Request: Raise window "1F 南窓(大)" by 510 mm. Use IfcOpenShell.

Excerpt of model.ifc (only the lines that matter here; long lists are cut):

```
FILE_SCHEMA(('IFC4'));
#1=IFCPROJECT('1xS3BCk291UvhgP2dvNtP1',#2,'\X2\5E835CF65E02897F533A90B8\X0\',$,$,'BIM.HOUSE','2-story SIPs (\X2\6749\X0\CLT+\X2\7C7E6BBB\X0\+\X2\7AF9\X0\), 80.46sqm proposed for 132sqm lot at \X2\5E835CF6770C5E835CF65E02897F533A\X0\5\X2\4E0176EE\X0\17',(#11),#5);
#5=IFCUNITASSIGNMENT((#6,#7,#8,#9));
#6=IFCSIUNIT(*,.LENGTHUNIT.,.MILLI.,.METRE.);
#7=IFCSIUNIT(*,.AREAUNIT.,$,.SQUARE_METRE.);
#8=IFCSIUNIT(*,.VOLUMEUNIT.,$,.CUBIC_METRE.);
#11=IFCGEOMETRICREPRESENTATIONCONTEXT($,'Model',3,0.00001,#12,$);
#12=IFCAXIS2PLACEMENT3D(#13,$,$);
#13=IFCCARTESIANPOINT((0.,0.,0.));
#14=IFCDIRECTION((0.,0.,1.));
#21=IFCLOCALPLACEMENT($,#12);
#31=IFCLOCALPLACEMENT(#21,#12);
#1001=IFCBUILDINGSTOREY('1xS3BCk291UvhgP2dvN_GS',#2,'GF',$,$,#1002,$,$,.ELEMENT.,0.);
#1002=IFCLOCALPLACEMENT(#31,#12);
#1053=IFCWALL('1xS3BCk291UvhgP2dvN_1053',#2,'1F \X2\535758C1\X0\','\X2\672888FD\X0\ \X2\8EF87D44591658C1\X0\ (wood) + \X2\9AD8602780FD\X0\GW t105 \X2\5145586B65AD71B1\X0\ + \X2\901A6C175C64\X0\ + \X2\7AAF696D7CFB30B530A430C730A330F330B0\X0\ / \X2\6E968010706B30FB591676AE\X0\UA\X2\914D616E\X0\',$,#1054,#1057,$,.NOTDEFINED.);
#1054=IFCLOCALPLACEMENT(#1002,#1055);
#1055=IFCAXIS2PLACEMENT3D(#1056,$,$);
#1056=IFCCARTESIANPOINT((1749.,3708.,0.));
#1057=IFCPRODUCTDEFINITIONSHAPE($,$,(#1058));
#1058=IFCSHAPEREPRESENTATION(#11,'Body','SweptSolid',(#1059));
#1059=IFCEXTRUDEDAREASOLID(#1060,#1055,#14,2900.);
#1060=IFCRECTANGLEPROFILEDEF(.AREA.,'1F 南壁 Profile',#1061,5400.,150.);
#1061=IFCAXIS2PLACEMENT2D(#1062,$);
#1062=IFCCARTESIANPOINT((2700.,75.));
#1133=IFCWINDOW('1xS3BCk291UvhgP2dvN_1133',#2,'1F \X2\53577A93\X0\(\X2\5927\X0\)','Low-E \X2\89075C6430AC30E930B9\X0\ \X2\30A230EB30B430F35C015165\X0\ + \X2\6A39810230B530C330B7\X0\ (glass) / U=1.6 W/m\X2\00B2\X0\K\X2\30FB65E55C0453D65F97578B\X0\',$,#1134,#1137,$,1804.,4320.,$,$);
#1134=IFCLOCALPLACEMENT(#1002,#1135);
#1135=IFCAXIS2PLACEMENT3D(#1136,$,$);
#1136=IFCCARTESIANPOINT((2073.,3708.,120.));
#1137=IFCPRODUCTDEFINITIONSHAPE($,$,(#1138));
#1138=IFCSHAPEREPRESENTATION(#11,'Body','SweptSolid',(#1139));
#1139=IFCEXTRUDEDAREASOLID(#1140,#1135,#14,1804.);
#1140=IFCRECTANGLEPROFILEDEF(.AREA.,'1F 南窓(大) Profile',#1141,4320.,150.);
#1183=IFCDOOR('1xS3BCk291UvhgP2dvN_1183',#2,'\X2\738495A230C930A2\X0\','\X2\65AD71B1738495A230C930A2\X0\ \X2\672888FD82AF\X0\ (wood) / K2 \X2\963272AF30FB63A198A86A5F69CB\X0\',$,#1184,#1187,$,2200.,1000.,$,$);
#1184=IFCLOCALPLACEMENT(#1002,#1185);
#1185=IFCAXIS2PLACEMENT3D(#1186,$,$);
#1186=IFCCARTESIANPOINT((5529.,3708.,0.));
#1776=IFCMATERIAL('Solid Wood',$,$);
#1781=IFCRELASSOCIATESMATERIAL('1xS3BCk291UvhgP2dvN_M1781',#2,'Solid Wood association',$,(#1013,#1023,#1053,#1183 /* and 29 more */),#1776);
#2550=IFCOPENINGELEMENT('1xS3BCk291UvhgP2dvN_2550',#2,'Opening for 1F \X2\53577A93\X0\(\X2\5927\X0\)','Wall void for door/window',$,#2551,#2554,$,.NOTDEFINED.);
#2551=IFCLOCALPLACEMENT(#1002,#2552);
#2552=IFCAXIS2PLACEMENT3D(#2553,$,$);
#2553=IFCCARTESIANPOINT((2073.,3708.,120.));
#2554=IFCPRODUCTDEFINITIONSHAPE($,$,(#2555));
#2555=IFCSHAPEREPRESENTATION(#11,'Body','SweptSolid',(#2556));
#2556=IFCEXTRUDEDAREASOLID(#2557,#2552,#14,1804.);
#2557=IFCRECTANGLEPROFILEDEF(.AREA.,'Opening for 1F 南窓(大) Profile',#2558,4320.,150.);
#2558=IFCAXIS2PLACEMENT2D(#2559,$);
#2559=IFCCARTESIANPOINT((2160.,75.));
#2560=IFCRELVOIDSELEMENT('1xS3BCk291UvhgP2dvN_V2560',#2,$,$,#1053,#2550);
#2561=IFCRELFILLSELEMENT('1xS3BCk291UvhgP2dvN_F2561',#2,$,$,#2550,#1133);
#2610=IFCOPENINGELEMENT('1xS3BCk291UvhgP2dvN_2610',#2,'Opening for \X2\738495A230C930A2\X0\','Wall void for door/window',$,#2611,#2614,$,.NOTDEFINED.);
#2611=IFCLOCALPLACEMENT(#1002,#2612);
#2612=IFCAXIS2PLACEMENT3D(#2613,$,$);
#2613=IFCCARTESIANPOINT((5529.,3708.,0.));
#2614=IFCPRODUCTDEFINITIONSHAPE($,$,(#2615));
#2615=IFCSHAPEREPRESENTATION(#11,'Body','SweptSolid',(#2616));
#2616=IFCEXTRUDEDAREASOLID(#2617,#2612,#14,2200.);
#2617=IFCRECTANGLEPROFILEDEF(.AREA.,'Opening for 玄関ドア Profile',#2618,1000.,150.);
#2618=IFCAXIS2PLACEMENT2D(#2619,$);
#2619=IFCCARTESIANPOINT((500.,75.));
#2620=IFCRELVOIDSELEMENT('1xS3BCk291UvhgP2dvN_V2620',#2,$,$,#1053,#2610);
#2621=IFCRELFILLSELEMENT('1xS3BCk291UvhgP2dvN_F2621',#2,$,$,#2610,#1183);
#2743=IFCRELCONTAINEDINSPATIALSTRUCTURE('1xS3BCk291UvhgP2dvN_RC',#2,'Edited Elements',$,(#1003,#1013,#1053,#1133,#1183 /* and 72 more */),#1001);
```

```python
import numpy as np
import ifcopenshell
import ifcopenshell.api.geometry
import ifcopenshell.util.placement
import ifcopenshell.util.unit

model = ifcopenshell.open("model.ifc")
unit_scale = ifcopenshell.util.unit.calculate_unit_scale(model)

window = model.by_guid("1xS3BCk291UvhgP2dvN_1133")
opening = window.FillsVoids[0].RelatingOpeningElement
dz = 510.0

shift = np.array([0.0, 0.0, dz])
# The window is not placed relative to its opening, so move both.
for product in (opening, window):
    matrix = ifcopenshell.util.placement.get_local_placement(product.ObjectPlacement)
    matrix[:3, 3] += shift
    ifcopenshell.api.geometry.edit_object_placement(model, product=product, matrix=matrix, is_si=False)

print(f"moved by {dz * unit_scale:+.3f} m")

model.write("model_updated.ifc")
```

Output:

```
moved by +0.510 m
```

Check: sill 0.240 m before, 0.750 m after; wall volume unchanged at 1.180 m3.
